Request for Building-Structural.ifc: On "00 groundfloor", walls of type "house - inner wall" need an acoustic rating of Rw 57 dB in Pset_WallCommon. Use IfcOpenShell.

First a look at what the model holds.

```python
import ifcopenshell
import ifcopenshell.util.element

model = ifcopenshell.open("Building-Structural.ifc")
print(model.schema)
storey = next(s for s in model.by_type("IfcBuildingStorey") if s.Name == "00 groundfloor")
walls = [e for e in ifcopenshell.util.element.get_decomposition(storey) if e.is_a("IfcWall")]
seen = {}
for e in walls:
    element_type = ifcopenshell.util.element.get_type(e)
    key = (element_type.Name if element_type != e and element_type else None, ifcopenshell.util.element.get_pset(e, "Pset_WallCommon", "AcousticRating"))
    seen[key] = seen.get(key, 0) + 1
for (name, value), count in sorted(seen.items(), key=str):
    print(count, "x", name, "|", value)
```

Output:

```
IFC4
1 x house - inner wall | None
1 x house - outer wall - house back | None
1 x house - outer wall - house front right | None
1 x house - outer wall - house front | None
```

```python
import ifcopenshell
import ifcopenshell.api.pset
import ifcopenshell.util.element

model = ifcopenshell.open("Building-Structural.ifc")

storey = next(s for s in model.by_type("IfcBuildingStorey") if s.Name == "00 groundfloor")
walls = [e for e in ifcopenshell.util.element.get_decomposition(storey) if e.is_a("IfcWall")]

count = 0
for e in walls:
    element_type = ifcopenshell.util.element.get_type(e)
    if element_type in (None, e) or element_type.Name != "house - inner wall":
        continue
    # add_pset returns the element's existing set when there is one.
    pset = ifcopenshell.api.pset.add_pset(model, product=e, name="Pset_WallCommon")
    ifcopenshell.api.pset.edit_pset(model, pset=pset, properties={"AcousticRating": "Rw 57 dB"})
    count += 1

print(count, "walls updated")

model.write("Building-Structural_edited.ifc")
```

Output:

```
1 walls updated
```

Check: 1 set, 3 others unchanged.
